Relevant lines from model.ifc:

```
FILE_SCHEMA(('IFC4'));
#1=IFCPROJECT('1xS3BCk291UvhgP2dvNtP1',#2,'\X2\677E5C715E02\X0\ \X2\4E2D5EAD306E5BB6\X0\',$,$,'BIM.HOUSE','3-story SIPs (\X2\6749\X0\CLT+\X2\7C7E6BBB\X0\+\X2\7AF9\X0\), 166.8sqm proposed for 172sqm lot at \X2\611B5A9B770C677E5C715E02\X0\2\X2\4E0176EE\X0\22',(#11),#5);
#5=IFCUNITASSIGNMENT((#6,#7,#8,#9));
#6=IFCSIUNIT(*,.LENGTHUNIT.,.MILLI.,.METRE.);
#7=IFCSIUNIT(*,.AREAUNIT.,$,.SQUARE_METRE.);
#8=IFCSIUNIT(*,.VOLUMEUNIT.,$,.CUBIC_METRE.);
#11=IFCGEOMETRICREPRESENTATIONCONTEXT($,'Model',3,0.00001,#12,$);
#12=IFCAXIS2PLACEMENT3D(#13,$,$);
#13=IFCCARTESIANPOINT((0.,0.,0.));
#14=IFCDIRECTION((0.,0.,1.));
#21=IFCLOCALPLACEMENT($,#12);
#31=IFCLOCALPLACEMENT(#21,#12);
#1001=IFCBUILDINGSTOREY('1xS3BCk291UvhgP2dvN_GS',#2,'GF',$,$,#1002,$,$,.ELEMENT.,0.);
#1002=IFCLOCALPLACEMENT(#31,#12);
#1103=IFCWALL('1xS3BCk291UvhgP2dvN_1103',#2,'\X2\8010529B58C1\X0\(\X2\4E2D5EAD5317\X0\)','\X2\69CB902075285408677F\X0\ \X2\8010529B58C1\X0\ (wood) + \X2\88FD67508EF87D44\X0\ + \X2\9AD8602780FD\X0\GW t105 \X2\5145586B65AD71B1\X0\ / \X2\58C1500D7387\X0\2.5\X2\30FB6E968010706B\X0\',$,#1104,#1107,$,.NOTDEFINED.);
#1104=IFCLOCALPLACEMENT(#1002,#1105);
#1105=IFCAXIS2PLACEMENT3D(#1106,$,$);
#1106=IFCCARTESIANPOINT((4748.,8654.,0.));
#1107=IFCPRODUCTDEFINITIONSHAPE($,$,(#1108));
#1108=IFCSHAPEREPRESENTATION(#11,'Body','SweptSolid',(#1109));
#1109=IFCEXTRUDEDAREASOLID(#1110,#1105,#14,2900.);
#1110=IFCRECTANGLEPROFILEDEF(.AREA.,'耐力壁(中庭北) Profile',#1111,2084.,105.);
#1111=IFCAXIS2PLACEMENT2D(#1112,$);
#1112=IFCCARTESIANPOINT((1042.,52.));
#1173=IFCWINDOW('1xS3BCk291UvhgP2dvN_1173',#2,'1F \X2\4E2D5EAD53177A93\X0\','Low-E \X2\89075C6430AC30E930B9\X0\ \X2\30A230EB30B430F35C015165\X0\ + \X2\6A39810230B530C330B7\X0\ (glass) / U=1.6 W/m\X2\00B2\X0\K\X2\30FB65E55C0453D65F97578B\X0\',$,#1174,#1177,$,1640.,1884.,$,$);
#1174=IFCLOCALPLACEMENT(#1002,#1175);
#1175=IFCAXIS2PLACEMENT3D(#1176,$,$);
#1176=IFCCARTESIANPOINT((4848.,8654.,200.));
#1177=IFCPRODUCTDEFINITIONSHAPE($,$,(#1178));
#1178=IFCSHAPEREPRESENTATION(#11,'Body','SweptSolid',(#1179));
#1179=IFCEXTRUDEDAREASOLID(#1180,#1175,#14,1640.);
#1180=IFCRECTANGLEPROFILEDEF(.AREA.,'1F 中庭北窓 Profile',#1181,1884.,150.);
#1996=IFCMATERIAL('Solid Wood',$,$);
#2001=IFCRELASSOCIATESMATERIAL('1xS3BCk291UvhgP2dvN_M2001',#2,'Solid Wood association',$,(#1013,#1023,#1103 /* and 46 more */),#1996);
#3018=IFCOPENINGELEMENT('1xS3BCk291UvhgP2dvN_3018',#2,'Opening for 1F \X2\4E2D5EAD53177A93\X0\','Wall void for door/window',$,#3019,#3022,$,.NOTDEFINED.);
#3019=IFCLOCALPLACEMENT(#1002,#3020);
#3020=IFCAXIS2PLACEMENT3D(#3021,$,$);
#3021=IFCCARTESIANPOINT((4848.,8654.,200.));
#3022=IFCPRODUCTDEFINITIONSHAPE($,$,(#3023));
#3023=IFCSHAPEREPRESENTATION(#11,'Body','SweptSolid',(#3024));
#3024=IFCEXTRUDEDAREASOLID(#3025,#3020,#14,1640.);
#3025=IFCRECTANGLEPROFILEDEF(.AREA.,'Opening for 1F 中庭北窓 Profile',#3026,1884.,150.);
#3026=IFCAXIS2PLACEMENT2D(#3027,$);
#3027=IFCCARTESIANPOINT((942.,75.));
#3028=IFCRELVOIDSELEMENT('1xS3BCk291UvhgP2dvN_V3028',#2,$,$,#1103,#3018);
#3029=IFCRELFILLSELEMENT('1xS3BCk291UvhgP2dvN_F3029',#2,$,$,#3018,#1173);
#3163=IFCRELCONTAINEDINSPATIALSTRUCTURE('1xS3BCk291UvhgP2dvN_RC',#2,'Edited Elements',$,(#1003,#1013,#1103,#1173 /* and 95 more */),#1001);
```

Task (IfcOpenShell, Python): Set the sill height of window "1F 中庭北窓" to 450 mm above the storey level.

```python
import numpy as np
import ifcopenshell
import ifcopenshell.api.geometry
import ifcopenshell.geom
import ifcopenshell.util.element
import ifcopenshell.util.placement
import ifcopenshell.util.shape
import ifcopenshell.util.unit

model = ifcopenshell.open("model.ifc")
unit_scale = ifcopenshell.util.unit.calculate_unit_scale(model)

window = model.by_guid("1xS3BCk291UvhgP2dvN_1173")
opening = window.FillsVoids[0].RelatingOpeningElement
storey = ifcopenshell.util.element.get_container(window, ifc_class="IfcBuildingStorey")
level = ifcopenshell.util.placement.get_local_placement(storey.ObjectPlacement)[2, 3]

# The opening's origin need not be at the sill, so measure its lowest point.
shape = ifcopenshell.geom.create_shape(ifcopenshell.geom.settings(), opening)
bottom = ifcopenshell.util.shape.get_shape_bottom_elevation(shape, shape.geometry) / unit_scale
dz = level + 450.0 - bottom

shift = np.array([0.0, 0.0, dz])
# The window is not placed relative to its opening, so move both.
for product in (opening, window):
    matrix = ifcopenshell.util.placement.get_local_placement(product.ObjectPlacement)
    matrix[:3, 3] += shift
    ifcopenshell.api.geometry.edit_object_placement(model, product=product, matrix=matrix, is_si=False)

print(f"moved by {dz * unit_scale:+.3f} m")

model.write("model_updated.ifc")
```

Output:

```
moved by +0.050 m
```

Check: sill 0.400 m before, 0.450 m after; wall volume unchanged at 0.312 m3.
